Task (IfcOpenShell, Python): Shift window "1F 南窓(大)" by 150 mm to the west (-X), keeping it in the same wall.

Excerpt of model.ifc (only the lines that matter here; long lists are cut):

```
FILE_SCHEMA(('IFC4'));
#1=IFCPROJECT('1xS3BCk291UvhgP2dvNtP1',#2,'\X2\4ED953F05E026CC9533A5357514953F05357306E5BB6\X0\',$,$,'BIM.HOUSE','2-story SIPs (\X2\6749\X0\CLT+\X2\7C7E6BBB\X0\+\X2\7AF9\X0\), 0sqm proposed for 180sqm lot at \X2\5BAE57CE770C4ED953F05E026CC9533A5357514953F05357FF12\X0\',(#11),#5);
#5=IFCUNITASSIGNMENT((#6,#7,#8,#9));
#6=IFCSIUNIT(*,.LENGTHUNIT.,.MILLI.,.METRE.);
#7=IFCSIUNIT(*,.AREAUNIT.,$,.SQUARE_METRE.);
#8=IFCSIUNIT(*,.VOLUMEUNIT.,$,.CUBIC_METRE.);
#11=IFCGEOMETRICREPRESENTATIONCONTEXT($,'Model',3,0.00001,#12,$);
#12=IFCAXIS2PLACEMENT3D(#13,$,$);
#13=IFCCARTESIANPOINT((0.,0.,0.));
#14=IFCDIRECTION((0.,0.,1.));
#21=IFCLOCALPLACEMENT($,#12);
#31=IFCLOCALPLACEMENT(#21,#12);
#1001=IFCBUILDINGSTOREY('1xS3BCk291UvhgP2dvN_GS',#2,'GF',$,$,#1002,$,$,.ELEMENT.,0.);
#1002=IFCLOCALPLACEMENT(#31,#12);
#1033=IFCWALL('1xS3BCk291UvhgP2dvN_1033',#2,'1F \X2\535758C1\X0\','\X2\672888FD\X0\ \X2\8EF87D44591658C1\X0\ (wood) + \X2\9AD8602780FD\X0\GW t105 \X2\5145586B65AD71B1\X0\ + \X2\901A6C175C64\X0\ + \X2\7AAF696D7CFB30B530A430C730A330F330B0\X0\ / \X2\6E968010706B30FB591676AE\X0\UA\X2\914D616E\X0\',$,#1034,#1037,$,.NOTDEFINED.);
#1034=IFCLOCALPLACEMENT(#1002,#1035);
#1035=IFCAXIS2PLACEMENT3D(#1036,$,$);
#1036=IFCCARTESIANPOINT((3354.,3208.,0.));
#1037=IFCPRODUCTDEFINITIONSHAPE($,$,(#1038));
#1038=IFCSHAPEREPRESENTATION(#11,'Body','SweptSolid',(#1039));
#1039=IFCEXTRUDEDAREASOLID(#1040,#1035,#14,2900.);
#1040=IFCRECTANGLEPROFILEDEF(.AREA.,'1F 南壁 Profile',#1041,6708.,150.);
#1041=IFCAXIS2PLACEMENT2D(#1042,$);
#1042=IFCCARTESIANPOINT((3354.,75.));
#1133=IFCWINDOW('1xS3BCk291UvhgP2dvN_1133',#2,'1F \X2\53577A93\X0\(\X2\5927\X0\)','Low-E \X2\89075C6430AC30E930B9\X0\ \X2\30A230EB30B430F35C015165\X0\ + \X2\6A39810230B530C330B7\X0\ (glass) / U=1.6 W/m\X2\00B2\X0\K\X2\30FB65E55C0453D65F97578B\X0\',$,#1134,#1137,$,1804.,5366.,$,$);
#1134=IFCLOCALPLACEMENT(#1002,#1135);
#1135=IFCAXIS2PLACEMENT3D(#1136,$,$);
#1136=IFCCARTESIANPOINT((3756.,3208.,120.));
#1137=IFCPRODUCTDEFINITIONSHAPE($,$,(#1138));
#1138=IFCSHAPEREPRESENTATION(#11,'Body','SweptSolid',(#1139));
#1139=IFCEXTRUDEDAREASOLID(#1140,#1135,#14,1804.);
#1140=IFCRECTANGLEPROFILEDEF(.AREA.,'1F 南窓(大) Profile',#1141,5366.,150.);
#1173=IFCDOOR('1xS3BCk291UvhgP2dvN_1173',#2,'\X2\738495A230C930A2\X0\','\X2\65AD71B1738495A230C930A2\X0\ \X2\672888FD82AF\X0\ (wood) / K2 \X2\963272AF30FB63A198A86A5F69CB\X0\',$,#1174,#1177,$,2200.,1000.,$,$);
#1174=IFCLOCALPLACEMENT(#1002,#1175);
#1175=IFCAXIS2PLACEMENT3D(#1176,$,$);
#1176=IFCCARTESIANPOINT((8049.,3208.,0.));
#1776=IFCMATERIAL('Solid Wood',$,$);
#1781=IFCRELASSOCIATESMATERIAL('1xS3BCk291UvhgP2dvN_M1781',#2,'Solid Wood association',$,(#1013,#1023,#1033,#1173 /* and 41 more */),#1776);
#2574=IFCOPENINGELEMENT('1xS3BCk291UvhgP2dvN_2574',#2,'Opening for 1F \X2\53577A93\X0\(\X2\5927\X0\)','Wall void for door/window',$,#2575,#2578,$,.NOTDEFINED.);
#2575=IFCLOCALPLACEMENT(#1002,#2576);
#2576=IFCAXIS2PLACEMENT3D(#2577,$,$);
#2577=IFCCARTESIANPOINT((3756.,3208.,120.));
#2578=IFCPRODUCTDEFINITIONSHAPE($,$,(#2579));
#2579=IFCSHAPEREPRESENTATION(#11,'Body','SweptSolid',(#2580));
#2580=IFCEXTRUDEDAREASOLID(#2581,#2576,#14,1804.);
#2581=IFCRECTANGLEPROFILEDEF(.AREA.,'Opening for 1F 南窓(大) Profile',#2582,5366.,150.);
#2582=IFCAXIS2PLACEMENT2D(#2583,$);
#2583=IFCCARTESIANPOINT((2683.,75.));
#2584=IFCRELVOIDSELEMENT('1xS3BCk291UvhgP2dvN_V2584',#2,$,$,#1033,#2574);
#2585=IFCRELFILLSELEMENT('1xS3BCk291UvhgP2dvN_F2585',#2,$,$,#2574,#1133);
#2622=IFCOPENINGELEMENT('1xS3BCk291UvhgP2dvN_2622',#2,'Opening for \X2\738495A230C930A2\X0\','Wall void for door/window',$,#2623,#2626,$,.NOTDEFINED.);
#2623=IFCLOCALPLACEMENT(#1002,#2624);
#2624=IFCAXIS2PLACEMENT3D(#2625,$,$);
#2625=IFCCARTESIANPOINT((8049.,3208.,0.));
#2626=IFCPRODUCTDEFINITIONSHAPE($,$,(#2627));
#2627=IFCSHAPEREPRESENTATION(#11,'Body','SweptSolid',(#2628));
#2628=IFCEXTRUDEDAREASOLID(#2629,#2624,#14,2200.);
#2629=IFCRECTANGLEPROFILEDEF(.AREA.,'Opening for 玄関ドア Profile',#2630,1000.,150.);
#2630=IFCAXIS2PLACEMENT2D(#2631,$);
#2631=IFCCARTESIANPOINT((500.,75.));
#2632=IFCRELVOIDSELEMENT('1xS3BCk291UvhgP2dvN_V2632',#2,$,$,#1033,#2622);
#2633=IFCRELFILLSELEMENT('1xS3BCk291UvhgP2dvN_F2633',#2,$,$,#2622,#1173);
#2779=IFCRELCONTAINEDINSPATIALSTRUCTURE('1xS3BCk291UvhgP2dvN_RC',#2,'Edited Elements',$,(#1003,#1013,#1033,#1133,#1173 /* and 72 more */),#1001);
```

```python
import ifcopenshell
import ifcopenshell.api.geometry
import ifcopenshell.util.placement
import ifcopenshell.util.unit

model = ifcopenshell.open("model.ifc")
unit_scale = ifcopenshell.util.unit.calculate_unit_scale(model)

window = model.by_id(1133)
opening = window.FillsVoids[0].RelatingOpeningElement
wall = opening.VoidsElements[0].RelatingBuildingElement

wall_matrix = ifcopenshell.util.placement.get_local_placement(wall.ObjectPlacement)
shift = wall_matrix[:3, 0] * -0.15 / unit_scale
before = ifcopenshell.util.placement.get_local_placement(window.ObjectPlacement)[:3, 3].copy()

# The window is not placed relative to its opening, so move both.
for product in (opening, window):
    matrix = ifcopenshell.util.placement.get_local_placement(product.ObjectPlacement)
    matrix[:3, 3] += shift
    ifcopenshell.api.geometry.edit_object_placement(model, product=product, matrix=matrix, is_si=False)

after = ifcopenshell.util.placement.get_local_placement(window.ObjectPlacement)[:3, 3]
print("window moved by", (after - before).round(3) + 0.0)

model.write("model-out.ifc")
```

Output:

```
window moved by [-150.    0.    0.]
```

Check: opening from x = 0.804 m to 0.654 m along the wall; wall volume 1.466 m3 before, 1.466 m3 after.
